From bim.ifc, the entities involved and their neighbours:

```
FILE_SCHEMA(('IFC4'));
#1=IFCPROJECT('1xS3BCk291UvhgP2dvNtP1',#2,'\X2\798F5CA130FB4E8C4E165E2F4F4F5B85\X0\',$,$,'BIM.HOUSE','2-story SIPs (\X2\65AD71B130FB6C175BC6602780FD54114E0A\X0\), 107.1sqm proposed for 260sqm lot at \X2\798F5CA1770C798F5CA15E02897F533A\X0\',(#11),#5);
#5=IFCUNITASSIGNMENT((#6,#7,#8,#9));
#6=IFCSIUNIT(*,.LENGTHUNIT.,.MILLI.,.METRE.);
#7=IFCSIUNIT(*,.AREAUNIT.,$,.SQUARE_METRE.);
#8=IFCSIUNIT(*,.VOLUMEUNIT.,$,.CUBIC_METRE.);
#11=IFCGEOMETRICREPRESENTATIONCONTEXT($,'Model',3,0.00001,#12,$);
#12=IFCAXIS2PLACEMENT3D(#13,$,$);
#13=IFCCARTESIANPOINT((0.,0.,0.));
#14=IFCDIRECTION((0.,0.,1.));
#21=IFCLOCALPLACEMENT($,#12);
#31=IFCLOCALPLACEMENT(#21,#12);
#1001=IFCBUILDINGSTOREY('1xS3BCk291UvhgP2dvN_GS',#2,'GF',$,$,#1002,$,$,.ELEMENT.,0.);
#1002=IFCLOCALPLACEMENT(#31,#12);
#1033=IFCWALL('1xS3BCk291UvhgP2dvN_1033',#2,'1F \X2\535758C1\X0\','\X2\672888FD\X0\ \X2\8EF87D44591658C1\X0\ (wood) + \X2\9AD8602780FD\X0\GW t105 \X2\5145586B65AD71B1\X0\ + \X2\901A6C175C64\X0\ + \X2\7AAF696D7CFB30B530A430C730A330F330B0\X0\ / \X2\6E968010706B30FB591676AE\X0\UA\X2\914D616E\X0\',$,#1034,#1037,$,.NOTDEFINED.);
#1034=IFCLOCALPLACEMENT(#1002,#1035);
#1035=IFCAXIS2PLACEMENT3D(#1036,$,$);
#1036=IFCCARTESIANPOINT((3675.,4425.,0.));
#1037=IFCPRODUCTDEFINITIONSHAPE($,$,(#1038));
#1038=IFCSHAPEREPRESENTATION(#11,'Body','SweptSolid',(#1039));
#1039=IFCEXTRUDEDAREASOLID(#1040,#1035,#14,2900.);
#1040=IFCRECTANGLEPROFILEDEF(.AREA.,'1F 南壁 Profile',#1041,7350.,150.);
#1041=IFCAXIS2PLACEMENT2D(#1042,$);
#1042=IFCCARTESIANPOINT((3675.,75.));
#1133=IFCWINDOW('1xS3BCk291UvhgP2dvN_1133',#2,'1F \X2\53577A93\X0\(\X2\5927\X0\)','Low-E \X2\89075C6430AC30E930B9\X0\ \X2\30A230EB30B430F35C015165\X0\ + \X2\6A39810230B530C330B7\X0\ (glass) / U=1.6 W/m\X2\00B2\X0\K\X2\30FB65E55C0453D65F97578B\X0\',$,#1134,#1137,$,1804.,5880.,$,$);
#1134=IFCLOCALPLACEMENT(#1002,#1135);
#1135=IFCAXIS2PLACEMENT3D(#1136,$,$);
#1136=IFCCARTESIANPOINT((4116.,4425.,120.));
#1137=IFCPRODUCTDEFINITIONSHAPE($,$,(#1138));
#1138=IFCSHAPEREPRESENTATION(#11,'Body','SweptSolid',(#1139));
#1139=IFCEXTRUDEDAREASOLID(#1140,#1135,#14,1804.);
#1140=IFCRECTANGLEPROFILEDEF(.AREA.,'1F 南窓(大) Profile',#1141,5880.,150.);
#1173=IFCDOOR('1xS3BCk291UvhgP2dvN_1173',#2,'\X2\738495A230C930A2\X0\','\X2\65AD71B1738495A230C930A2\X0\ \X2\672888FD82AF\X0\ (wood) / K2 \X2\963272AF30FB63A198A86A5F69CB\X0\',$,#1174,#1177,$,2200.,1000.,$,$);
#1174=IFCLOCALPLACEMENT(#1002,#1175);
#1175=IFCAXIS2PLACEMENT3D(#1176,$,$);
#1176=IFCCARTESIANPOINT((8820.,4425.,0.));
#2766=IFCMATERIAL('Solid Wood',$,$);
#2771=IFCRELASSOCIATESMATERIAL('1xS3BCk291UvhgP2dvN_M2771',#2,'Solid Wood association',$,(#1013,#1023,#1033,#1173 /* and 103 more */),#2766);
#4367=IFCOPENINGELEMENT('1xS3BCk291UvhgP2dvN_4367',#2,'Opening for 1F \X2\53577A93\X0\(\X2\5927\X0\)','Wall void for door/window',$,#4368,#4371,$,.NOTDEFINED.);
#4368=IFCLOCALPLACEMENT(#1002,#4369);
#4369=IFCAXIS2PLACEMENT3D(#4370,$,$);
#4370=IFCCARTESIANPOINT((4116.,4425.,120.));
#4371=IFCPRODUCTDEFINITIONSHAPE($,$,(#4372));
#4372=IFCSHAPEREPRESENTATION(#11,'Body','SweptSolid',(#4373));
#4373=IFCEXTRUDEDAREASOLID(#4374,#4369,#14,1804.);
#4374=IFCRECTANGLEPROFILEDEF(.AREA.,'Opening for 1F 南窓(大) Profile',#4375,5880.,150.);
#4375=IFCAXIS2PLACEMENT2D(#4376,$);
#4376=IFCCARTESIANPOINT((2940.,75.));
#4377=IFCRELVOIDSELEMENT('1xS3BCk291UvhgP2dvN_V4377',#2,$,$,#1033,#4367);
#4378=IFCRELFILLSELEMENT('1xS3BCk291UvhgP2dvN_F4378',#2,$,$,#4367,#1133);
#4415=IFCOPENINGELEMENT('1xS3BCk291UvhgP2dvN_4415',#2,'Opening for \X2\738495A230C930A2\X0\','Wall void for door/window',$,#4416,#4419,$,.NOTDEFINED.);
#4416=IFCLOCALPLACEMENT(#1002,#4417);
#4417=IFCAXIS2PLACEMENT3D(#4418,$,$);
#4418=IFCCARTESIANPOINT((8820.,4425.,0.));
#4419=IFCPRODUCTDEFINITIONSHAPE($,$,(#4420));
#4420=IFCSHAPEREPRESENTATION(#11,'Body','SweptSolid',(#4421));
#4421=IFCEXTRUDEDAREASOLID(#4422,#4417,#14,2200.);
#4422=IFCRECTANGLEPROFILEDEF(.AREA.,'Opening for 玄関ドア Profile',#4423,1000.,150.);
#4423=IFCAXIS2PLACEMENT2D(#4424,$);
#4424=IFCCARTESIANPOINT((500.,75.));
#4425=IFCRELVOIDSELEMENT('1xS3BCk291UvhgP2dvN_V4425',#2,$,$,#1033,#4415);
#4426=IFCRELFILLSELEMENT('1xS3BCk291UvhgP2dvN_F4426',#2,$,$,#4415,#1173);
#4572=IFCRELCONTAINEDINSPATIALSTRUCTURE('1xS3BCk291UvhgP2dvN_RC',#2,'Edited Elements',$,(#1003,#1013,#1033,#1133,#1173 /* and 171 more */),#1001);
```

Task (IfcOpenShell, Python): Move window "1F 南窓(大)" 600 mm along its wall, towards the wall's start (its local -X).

```python
import ifcopenshell
import ifcopenshell.api.geometry
import ifcopenshell.util.placement

model = ifcopenshell.open("bim.ifc")

window = model.by_guid("1xS3BCk291UvhgP2dvN_1133")
opening = window.FillsVoids[0].RelatingOpeningElement
wall = opening.VoidsElements[0].RelatingBuildingElement

wall_matrix = ifcopenshell.util.placement.get_local_placement(wall.ObjectPlacement)
shift = wall_matrix[:3, 0] * -600.0
before = ifcopenshell.util.placement.get_local_placement(window.ObjectPlacement)[:3, 3].copy()

# The window is not placed relative to its opening, so move both.
for product in (opening, window):
    matrix = ifcopenshell.util.placement.get_local_placement(product.ObjectPlacement)
    matrix[:3, 3] += shift
    ifcopenshell.api.geometry.edit_object_placement(model, product=product, matrix=matrix, is_si=False)

after = ifcopenshell.util.placement.get_local_placement(window.ObjectPlacement)[:3, 3]
print("window moved by", (after - before).round(3) + 0.0)

model.write("bim_rev.ifc")
```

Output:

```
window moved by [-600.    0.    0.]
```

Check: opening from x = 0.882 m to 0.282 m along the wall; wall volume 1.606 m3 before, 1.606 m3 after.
